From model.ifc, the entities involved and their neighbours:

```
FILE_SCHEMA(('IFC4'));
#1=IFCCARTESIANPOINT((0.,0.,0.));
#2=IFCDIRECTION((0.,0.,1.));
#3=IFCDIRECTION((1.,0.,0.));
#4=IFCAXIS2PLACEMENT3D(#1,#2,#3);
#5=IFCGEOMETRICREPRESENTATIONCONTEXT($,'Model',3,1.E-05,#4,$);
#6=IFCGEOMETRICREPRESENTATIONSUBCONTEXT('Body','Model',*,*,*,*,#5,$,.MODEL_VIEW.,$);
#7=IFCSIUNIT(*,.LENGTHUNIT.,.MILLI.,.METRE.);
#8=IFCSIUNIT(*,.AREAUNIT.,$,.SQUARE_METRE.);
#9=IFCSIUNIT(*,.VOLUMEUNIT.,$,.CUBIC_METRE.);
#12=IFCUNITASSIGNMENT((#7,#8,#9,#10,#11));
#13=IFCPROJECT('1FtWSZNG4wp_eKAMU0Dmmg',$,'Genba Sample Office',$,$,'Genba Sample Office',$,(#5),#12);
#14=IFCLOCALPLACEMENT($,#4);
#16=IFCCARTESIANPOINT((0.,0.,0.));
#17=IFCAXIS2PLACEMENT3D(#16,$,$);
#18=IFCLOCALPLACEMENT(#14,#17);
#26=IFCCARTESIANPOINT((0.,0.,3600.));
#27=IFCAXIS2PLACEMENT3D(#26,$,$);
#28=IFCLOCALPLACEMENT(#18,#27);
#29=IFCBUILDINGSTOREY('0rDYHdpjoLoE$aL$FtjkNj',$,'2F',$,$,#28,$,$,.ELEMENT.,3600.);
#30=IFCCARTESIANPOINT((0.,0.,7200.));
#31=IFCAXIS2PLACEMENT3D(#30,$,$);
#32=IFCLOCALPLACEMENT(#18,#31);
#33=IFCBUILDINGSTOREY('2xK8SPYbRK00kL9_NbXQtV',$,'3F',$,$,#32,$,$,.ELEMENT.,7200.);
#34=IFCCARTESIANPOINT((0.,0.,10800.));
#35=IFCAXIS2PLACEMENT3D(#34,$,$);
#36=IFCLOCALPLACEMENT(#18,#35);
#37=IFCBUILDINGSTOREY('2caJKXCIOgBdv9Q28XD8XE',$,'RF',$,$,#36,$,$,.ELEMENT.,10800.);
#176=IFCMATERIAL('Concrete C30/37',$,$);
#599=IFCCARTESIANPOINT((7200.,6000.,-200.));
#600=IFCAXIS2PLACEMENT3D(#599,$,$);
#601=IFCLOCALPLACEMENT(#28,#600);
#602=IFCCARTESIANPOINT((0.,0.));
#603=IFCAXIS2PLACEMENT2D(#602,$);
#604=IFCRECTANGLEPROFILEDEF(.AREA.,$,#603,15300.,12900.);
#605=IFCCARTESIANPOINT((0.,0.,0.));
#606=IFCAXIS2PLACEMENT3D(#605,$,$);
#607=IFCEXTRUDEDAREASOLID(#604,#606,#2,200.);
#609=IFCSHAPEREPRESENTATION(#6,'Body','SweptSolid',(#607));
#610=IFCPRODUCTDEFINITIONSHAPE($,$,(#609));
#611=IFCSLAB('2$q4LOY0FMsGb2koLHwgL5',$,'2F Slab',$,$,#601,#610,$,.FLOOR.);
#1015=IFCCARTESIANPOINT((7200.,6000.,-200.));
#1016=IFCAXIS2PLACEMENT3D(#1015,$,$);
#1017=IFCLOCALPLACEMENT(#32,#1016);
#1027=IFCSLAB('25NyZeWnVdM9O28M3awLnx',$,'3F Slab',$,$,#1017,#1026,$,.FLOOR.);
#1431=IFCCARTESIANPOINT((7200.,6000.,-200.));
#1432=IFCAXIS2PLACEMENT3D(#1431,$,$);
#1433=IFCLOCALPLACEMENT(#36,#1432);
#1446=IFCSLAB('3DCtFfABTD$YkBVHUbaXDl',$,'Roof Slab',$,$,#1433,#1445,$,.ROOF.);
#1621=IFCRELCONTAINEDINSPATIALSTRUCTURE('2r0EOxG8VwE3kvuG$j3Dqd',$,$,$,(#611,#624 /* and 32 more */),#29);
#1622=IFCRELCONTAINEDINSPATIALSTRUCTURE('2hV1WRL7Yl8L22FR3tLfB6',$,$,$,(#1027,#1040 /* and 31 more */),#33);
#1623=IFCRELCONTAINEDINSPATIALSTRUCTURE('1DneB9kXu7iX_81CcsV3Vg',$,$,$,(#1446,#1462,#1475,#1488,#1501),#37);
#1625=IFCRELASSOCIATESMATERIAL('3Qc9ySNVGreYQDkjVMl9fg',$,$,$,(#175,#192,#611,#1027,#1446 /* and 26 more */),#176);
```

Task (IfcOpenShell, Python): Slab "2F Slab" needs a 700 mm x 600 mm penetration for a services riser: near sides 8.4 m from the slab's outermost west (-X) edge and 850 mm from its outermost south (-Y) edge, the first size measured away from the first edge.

```python
import numpy as np
import ifcopenshell
import ifcopenshell.api.feature
import ifcopenshell.api.geometry
import ifcopenshell.api.root
import ifcopenshell.geom
import ifcopenshell.util.placement
import ifcopenshell.util.representation
import ifcopenshell.util.shape
import ifcopenshell.util.unit

model = ifcopenshell.open("model.ifc")
unit_scale = ifcopenshell.util.unit.calculate_unit_scale(model)
settings = ifcopenshell.geom.settings()


def volume(element):
    """Net volume in cubic metres, openings subtracted."""
    shape = ifcopenshell.geom.create_shape(settings, element)
    return ifcopenshell.util.shape.get_volume(shape.geometry)


slab = model.by_guid("2$q4LOY0FMsGb2koLHwgL5")
before = volume(slab)

# Extent in the slab's own axes, in metres. The edges named are its -X and -Y sides.
slab_shape = ifcopenshell.geom.create_shape(settings, slab)
vertices = ifcopenshell.util.shape.get_vertices(slab_shape.geometry)
x_min, y_min, bottom = vertices.min(axis=0)
top = vertices[:, 2].max()

opening = ifcopenshell.api.root.create_entity(model, ifc_class="IfcOpeningElement", name="Services riser opening", predefined_type="OPENING")
context = ifcopenshell.util.representation.get_context(model, "Model", "Body", "MODEL_VIEW")
width, depth = 0.7, 0.6
outline = [(0.0, 0.0), (width, 0.0), (width, depth), (0.0, depth), (0.0, 0.0)]
# Overshoot both faces by 50 mm so the cut is clean.
shape = ifcopenshell.api.geometry.add_slab_representation(
    model, context=context, depth=top - bottom + 0.1, polyline=outline
)
ifcopenshell.api.geometry.assign_representation(model, product=opening, representation=shape)

matrix = ifcopenshell.util.placement.get_local_placement(slab.ObjectPlacement)
matrix[:, 3] = matrix @ np.append(np.array([x_min + 8.4, y_min + 0.85, bottom - 0.05]) / unit_scale, 1.0)
ifcopenshell.api.geometry.edit_object_placement(model, product=opening, matrix=matrix, is_si=False)
ifcopenshell.api.feature.add_feature(model, feature=opening, element=slab)

after = volume(slab)

print(f"slab volume {before:.3f} -> {after:.3f} m3")

model.write("model_v2.ifc")
```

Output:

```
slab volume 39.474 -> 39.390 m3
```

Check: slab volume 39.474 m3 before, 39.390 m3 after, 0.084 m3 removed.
